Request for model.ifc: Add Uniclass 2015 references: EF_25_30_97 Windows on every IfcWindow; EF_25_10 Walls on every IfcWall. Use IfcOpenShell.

First a look at what the model holds.

```python
import ifcopenshell

model = ifcopenshell.open("model.ifc")
print(model.schema)
print("classifications:", [c.Name for c in model.by_type("IfcClassification")])
for ifc_class in ("IfcDoor", "IfcRoof", "IfcStair", "IfcWall", "IfcWindow"):
    print(ifc_class, len(model.by_type(ifc_class)))
```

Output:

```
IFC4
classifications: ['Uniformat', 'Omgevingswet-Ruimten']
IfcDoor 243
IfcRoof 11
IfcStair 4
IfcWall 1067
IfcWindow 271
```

```python
import ifcopenshell
import ifcopenshell.api.classification

model = ifcopenshell.open("model.ifc")

system = ifcopenshell.api.classification.add_classification(model, classification="Uniclass 2015")

codes = {
    "IfcWindow": ("EF_25_30_97", "Windows"),
    "IfcWall": ("EF_25_10", "Walls"),
}
for ifc_class, (code, name) in codes.items():
    products = model.by_type(ifc_class)
    ifcopenshell.api.classification.add_reference(
        model, products=products, classification=system, identification=code, name=name
    )
    print(code, len(products))

model.write("model-out.ifc")
```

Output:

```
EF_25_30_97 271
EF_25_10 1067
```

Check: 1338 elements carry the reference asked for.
